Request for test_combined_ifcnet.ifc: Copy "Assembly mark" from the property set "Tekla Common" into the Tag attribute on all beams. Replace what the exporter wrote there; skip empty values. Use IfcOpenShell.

First a look at what the model holds.

```python
import ifcopenshell
import ifcopenshell.util.element

model = ifcopenshell.open("test_combined_ifcnet.ifc")
print(model.schema)
beams = model.by_type("IfcBeam")
print(len(beams), "beams")
for e in beams[:8]:
    source = ifcopenshell.util.element.get_pset(e, "Tekla Common", "Assembly mark")
    target = e.Tag
    print(e.id(), repr(source), repr(target), sep=" | ")
```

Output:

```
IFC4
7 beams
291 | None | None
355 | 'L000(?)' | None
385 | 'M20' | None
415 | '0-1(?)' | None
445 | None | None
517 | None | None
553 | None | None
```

```python
import ifcopenshell
import ifcopenshell.util.element

model = ifcopenshell.open("test_combined_ifcnet.ifc")

count = 0
for e in model.by_type("IfcBeam"):
    value = ifcopenshell.util.element.get_pset(e, "Tekla Common", "Assembly mark")
    current = e.Tag
    if not value or not value.strip() or current == value:
        continue
    e.Tag = value
    count += 1

print(count, "beams updated")

model.write("test_combined_ifcnet-out.ifc")
```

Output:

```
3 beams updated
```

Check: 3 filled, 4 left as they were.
